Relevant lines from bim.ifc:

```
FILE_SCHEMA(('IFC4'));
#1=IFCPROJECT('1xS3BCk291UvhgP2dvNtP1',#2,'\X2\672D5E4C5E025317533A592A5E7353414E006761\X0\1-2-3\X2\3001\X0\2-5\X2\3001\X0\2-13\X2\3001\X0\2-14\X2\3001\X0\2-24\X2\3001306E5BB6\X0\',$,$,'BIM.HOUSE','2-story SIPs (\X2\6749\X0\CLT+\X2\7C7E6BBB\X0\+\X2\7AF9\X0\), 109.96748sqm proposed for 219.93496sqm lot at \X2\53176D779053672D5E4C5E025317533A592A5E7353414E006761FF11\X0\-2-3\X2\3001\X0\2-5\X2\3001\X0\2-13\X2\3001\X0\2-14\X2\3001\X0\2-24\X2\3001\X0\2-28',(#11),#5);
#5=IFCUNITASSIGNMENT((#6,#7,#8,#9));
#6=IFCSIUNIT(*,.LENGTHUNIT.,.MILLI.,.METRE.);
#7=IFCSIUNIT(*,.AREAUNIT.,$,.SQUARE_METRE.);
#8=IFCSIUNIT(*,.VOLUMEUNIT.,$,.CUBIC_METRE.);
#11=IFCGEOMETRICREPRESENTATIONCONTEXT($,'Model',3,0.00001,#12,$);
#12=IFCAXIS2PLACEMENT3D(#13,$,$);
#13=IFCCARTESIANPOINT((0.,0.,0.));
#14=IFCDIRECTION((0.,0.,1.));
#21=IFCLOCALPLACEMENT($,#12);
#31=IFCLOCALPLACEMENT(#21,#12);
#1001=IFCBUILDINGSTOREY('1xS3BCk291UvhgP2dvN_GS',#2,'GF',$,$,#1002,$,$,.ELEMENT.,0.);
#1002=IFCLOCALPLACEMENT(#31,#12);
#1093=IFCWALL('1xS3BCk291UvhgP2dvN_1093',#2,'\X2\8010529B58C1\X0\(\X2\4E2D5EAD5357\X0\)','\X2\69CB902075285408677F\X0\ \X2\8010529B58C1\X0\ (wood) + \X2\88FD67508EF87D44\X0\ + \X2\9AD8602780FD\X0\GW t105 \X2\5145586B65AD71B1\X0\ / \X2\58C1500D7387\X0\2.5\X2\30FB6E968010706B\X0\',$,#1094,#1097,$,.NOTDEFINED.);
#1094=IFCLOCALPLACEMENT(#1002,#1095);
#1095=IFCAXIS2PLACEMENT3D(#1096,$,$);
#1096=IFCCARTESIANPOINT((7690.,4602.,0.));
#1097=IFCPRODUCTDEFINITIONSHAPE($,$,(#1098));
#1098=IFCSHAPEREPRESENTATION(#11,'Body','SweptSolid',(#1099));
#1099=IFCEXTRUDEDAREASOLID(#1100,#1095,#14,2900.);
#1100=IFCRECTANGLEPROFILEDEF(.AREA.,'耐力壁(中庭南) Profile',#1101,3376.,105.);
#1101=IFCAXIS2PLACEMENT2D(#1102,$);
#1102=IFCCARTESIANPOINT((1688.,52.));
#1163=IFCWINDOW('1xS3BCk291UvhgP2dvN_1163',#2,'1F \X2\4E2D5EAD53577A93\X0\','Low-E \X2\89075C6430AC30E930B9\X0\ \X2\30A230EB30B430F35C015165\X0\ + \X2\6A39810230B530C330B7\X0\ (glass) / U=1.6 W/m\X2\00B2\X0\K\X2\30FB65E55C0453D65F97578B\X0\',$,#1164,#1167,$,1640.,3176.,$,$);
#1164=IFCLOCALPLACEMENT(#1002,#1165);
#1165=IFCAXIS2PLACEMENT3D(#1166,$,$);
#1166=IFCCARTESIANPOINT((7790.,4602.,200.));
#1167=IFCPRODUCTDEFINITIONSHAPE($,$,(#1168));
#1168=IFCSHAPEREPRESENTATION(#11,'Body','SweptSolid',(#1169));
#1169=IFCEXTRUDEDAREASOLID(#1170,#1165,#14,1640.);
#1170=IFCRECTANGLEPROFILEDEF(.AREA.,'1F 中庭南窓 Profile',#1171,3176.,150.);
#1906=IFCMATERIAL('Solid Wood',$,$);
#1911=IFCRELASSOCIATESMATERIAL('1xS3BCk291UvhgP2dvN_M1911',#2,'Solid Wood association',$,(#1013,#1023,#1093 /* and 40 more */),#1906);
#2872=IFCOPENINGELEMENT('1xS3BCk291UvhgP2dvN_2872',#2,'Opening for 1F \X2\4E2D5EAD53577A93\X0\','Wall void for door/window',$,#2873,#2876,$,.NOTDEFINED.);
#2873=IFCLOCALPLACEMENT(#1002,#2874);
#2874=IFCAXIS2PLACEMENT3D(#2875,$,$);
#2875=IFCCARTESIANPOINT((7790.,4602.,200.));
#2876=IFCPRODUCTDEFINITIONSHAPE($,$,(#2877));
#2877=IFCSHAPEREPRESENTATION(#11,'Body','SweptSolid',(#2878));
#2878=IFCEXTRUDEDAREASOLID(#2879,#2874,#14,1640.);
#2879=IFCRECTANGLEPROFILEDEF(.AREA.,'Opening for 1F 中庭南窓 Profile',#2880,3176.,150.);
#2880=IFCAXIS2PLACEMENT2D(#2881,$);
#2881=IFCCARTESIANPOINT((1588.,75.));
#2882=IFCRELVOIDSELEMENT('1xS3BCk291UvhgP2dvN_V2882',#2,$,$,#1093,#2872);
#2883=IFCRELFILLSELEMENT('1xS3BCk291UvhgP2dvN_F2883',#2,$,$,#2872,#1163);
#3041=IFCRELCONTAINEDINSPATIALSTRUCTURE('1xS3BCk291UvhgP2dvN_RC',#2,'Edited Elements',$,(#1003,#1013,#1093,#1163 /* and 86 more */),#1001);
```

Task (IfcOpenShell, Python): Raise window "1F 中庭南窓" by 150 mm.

```python
import numpy as np
import ifcopenshell
import ifcopenshell.api.geometry
import ifcopenshell.util.placement
import ifcopenshell.util.unit

model = ifcopenshell.open("bim.ifc")
unit_scale = ifcopenshell.util.unit.calculate_unit_scale(model)

window = model.by_guid("1xS3BCk291UvhgP2dvN_1163")
opening = window.FillsVoids[0].RelatingOpeningElement
dz = 0.15 / unit_scale

shift = np.array([0.0, 0.0, dz])
# The window is not placed relative to its opening, so move both.
for product in (opening, window):
    matrix = ifcopenshell.util.placement.get_local_placement(product.ObjectPlacement)
    matrix[:3, 3] += shift
    ifcopenshell.api.geometry.edit_object_placement(model, product=product, matrix=matrix, is_si=False)

print(f"moved by {dz * unit_scale:+.3f} m")

model.write("bim_rev.ifc")
```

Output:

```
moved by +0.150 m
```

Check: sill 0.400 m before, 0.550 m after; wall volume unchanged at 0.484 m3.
